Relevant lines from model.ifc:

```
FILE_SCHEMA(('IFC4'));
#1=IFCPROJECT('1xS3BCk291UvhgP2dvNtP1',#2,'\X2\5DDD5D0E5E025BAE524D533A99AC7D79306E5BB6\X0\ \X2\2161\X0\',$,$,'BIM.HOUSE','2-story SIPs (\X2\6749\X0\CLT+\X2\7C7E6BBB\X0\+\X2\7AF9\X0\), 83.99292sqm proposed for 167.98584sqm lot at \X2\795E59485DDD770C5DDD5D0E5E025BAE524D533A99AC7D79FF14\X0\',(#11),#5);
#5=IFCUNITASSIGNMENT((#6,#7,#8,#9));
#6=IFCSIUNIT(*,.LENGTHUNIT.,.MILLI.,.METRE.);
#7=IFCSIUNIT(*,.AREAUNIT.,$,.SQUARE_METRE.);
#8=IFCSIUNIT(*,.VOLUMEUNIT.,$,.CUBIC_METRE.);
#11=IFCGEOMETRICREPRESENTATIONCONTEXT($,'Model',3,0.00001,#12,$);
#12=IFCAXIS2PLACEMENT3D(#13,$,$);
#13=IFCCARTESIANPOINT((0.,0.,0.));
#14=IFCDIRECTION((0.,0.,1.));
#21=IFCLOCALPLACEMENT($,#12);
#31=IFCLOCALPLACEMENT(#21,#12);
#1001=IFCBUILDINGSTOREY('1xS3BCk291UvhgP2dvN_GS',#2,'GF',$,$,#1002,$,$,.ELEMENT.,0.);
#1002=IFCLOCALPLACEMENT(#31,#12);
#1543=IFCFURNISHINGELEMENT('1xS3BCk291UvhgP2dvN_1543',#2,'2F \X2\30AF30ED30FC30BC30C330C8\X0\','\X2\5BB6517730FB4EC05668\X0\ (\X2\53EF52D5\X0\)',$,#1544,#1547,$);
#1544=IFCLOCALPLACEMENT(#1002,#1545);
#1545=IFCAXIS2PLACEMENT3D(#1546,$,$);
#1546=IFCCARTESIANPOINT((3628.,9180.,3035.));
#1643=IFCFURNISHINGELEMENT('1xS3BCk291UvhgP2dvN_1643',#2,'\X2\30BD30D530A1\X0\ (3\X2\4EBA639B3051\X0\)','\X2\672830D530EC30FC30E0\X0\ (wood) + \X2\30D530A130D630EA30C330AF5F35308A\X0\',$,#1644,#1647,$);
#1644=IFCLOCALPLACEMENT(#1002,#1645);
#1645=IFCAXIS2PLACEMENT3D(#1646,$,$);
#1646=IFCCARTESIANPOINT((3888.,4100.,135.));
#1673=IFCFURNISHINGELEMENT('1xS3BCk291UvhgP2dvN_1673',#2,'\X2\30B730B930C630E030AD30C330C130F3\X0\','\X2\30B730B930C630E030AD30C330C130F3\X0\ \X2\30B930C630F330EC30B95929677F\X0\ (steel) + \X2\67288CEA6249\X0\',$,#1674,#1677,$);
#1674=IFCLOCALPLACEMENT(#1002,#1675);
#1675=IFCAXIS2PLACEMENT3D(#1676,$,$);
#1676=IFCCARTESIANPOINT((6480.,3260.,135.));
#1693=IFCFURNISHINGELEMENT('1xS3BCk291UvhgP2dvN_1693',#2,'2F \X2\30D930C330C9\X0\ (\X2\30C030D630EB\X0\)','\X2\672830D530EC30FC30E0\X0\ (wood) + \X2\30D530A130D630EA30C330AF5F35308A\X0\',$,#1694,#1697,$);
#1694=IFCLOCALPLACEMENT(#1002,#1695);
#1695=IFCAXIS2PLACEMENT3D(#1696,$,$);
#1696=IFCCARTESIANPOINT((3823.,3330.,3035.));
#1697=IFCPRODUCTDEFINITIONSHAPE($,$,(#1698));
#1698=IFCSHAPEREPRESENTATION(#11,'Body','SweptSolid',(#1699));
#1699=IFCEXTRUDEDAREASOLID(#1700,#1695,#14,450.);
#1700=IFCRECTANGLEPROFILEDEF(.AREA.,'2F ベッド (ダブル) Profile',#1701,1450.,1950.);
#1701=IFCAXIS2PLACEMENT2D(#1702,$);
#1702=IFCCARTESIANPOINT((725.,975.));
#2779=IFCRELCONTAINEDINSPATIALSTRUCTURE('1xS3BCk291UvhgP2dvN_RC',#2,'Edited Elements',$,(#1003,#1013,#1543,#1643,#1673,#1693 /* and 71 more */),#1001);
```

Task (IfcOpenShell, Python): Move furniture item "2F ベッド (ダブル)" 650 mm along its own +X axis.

```python
import ifcopenshell
import ifcopenshell.api.geometry
import ifcopenshell.util.placement

model = ifcopenshell.open("model.ifc")

item = model.by_guid("1xS3BCk291UvhgP2dvN_1693")
matrix = ifcopenshell.util.placement.get_local_placement(item.ObjectPlacement)
matrix[:3, 3] += matrix[:3, 0] * 650.0
ifcopenshell.api.geometry.edit_object_placement(model, product=item, matrix=matrix, is_si=False)

print(ifcopenshell.util.placement.get_local_placement(item.ObjectPlacement).round(3) + 0.0)

model.write("model_edited.ifc")
```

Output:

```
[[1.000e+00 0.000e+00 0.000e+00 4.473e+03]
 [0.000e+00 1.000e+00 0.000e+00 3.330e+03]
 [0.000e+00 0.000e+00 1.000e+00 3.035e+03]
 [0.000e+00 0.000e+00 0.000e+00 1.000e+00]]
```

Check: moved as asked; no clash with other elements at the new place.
